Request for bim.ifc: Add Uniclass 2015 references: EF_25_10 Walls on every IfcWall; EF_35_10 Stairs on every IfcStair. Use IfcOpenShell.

First a look at what the model holds.

```python
import ifcopenshell

model = ifcopenshell.open("bim.ifc")
print(model.schema)
print("classifications:", [c.Name for c in model.by_type("IfcClassification")])
for ifc_class in ("IfcDoor", "IfcRoof", "IfcStair", "IfcWall", "IfcWindow"):
    print(ifc_class, len(model.by_type(ifc_class)))
```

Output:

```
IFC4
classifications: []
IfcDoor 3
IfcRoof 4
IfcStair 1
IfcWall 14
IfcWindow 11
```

```python
import ifcopenshell
import ifcopenshell.api.classification

model = ifcopenshell.open("bim.ifc")

system = ifcopenshell.api.classification.add_classification(model, classification="Uniclass 2015")

codes = {
    "IfcWall": ("EF_25_10", "Walls"),
    "IfcStair": ("EF_35_10", "Stairs"),
}
for ifc_class, (code, name) in codes.items():
    products = model.by_type(ifc_class)
    ifcopenshell.api.classification.add_reference(
        model, products=products, classification=system, identification=code, name=name
    )
    print(code, len(products))

model.write("bim_rev.ifc")
```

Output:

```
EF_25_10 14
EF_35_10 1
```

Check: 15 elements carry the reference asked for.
